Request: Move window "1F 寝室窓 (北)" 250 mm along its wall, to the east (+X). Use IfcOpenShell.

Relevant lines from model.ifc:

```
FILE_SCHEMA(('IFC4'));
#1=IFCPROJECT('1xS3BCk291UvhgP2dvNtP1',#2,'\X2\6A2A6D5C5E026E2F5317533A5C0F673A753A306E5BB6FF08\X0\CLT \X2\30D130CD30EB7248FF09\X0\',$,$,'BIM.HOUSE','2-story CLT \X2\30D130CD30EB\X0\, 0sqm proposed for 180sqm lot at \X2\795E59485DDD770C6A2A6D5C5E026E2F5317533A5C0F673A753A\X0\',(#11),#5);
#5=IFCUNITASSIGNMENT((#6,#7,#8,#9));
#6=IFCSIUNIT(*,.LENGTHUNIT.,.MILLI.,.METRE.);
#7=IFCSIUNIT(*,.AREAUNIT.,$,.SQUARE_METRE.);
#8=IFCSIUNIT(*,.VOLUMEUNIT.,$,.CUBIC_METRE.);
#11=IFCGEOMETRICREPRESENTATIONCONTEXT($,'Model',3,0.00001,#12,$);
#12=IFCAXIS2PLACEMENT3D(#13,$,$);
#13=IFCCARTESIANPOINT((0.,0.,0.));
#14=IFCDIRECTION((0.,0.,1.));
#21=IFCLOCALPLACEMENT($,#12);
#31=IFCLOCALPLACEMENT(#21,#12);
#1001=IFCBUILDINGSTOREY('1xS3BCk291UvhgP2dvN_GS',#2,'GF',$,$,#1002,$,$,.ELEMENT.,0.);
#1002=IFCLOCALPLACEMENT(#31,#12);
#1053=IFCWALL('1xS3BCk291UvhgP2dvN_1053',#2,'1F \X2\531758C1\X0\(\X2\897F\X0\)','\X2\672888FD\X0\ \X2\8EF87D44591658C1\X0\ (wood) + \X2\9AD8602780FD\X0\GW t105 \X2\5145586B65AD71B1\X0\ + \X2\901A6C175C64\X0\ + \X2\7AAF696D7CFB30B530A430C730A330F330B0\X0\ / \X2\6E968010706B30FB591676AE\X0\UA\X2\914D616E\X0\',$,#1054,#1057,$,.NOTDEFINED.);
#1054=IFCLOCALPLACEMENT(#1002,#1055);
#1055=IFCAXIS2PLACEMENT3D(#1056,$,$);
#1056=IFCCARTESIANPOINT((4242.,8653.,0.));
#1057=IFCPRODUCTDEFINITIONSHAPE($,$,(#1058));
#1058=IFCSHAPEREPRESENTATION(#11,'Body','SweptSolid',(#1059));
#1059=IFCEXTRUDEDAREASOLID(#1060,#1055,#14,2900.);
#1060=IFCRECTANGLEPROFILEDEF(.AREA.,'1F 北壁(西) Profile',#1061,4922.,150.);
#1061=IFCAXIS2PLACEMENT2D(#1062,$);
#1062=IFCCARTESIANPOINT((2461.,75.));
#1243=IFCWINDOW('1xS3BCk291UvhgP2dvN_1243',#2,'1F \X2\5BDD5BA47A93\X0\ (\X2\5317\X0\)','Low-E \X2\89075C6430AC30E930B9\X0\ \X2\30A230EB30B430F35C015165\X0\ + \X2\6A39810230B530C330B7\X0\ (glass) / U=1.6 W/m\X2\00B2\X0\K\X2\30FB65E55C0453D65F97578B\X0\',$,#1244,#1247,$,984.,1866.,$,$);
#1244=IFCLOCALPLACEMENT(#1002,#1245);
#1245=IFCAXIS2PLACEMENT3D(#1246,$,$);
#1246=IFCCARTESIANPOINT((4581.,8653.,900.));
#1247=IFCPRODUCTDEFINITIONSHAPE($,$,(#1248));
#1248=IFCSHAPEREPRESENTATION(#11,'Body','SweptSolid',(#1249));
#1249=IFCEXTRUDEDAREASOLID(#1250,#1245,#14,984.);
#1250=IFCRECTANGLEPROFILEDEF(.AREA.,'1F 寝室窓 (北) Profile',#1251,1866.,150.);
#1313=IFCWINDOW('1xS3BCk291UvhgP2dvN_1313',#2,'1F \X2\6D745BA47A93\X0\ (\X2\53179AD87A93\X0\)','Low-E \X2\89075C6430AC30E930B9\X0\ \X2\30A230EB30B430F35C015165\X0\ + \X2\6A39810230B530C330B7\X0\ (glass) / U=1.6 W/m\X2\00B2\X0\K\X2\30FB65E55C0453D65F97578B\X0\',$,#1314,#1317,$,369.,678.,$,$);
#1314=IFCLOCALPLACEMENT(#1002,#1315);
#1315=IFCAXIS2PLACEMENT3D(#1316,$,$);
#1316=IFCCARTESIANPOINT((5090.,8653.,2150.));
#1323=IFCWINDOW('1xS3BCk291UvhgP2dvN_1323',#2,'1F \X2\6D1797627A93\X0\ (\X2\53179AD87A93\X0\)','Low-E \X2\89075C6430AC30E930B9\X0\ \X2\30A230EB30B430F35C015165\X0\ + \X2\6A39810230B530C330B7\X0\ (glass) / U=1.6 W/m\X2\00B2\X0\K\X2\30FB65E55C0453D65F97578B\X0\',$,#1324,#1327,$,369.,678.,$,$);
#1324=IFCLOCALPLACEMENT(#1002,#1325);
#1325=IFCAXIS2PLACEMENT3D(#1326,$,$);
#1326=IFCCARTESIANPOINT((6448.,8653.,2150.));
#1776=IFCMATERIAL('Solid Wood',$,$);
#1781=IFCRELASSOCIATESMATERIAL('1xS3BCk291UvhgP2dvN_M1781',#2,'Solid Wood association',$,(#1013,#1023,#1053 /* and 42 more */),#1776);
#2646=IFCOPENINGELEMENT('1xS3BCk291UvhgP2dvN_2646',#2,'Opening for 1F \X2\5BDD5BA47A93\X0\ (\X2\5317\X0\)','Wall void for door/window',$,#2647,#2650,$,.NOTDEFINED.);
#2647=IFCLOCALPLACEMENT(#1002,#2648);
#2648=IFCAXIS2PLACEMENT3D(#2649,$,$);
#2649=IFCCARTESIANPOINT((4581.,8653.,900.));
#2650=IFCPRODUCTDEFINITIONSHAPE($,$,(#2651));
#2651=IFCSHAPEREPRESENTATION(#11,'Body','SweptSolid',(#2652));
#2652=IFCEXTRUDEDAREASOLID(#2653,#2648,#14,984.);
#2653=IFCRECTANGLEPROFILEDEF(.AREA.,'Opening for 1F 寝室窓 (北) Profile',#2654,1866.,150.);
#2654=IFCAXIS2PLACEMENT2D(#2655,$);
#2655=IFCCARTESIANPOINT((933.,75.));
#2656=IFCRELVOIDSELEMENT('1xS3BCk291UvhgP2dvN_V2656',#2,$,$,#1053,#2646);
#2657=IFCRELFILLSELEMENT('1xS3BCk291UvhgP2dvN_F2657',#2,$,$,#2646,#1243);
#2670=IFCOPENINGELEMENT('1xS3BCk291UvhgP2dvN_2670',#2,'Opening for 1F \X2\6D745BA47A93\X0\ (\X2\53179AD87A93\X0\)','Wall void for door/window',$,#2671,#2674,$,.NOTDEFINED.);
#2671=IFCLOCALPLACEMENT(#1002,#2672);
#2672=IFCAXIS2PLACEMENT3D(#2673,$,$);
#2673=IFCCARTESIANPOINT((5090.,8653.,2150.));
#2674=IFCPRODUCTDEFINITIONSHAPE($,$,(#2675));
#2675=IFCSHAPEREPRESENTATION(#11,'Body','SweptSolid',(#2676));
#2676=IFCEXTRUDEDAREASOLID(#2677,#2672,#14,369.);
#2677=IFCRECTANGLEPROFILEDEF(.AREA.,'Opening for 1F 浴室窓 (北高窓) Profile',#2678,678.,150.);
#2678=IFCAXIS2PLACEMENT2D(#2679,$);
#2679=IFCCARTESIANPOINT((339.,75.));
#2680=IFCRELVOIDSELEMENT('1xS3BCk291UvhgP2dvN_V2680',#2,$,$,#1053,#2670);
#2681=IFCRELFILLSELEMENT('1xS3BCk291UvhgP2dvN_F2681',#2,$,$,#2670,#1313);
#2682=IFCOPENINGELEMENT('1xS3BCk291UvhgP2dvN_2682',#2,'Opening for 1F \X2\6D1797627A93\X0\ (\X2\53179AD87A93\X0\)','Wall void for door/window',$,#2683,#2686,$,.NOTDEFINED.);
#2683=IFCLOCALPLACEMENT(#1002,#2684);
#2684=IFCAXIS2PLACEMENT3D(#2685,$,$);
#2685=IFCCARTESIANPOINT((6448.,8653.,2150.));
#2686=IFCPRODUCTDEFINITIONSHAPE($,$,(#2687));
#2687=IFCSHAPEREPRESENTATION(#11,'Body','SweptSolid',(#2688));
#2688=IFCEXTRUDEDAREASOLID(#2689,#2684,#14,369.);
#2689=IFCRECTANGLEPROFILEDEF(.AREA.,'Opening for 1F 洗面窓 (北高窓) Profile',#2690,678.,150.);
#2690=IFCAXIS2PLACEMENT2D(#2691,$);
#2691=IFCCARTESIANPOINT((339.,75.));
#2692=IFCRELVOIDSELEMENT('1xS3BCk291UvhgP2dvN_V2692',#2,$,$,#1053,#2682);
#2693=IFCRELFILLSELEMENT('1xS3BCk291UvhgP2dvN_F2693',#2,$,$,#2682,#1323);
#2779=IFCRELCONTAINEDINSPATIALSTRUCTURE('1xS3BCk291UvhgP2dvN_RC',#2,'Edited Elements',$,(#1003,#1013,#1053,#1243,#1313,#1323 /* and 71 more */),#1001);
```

```python
import ifcopenshell
import ifcopenshell.api.geometry
import ifcopenshell.util.placement
import ifcopenshell.util.unit

model = ifcopenshell.open("model.ifc")
unit_scale = ifcopenshell.util.unit.calculate_unit_scale(model)

window = model.by_guid("1xS3BCk291UvhgP2dvN_1243")
opening = window.FillsVoids[0].RelatingOpeningElement
wall = opening.VoidsElements[0].RelatingBuildingElement

wall_matrix = ifcopenshell.util.placement.get_local_placement(wall.ObjectPlacement)
shift = wall_matrix[:3, 0] * 0.25 / unit_scale
before = ifcopenshell.util.placement.get_local_placement(window.ObjectPlacement)[:3, 3].copy()

# The window is not placed relative to its opening, so move both.
for product in (opening, window):
    matrix = ifcopenshell.util.placement.get_local_placement(product.ObjectPlacement)
    matrix[:3, 3] += shift
    ifcopenshell.api.geometry.edit_object_placement(model, product=product, matrix=matrix, is_si=False)

after = ifcopenshell.util.placement.get_local_placement(window.ObjectPlacement)[:3, 3]
print("window moved by", (after - before).round(3) + 0.0)

model.write("model_updated.ifc")
```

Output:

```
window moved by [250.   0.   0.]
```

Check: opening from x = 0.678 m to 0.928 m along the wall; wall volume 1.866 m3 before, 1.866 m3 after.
